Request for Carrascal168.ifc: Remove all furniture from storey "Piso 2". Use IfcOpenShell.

First a look at what the model holds.

```python
import ifcopenshell
import ifcopenshell.util.element

model = ifcopenshell.open("Carrascal168.ifc")
print(model.schema)
storey = next(s for s in model.by_type("IfcBuildingStorey") if s.Name == "Piso 2")
furniture = [e for e in ifcopenshell.util.element.get_decomposition(storey) if e.is_a("IfcFurnishingElement")]
seen = {}
for e in furniture:
    element_type = ifcopenshell.util.element.get_type(e)
    name = element_type.Name if element_type not in (None, e) else None
    seen[name] = seen.get(name, 0) + 1
for name, count in sorted(seen.items(), key=str):
    print(count, "x", name)
```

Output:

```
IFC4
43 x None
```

```python
import ifcopenshell
import ifcopenshell.api.root
import ifcopenshell.util.element

model = ifcopenshell.open("Carrascal168.ifc")

storey = next(s for s in model.by_type("IfcBuildingStorey") if s.Name == "Piso 2")
furniture = [e for e in ifcopenshell.util.element.get_decomposition(storey) if e.is_a("IfcFurnishingElement")]

for e in furniture:
    ifcopenshell.api.root.remove_product(model, product=e)
print(len(furniture), "removed")

model.write("Carrascal168_rev.ifc")
```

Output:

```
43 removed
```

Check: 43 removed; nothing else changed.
